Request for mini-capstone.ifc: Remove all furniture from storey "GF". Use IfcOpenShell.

First a look at what the model holds.

```python
import ifcopenshell
import ifcopenshell.util.element

model = ifcopenshell.open("mini-capstone.ifc")
print(model.schema)
storey = next(s for s in model.by_type("IfcBuildingStorey") if s.Name == "GF")
furniture = [e for e in ifcopenshell.util.element.get_decomposition(storey) if e.is_a("IfcFurnishingElement")]
seen = {}
for e in furniture:
    element_type = ifcopenshell.util.element.get_type(e)
    name = element_type.Name if element_type not in (None, e) else None
    seen[name] = seen.get(name, 0) + 1
for name, count in sorted(seen.items(), key=str):
    print(count, "x", name)
```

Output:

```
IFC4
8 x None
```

```python
import ifcopenshell
import ifcopenshell.api.root
import ifcopenshell.util.element

model = ifcopenshell.open("mini-capstone.ifc")

storey = next(s for s in model.by_type("IfcBuildingStorey") if s.Name == "GF")
furniture = [e for e in ifcopenshell.util.element.get_decomposition(storey) if e.is_a("IfcFurnishingElement")]

for e in furniture:
    ifcopenshell.api.root.remove_product(model, product=e)
print(len(furniture), "removed")

model.write("mini-capstone-out.ifc")
```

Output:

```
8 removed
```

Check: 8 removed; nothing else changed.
